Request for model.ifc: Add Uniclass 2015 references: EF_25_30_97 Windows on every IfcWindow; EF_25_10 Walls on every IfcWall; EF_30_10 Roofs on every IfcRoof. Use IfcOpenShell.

First a look at what the model holds.

```python
import ifcopenshell

model = ifcopenshell.open("model.ifc")
print(model.schema)
print("classifications:", [c.Name for c in model.by_type("IfcClassification")])
for ifc_class in ("IfcDoor", "IfcRoof", "IfcStair", "IfcWall", "IfcWindow"):
    print(ifc_class, len(model.by_type(ifc_class)))
```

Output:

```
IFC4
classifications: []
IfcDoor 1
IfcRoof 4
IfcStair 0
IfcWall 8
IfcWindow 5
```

```python
import ifcopenshell
import ifcopenshell.api.classification

model = ifcopenshell.open("model.ifc")

system = ifcopenshell.api.classification.add_classification(model, classification="Uniclass 2015")

codes = {
    "IfcWindow": ("EF_25_30_97", "Windows"),
    "IfcWall": ("EF_25_10", "Walls"),
    "IfcRoof": ("EF_30_10", "Roofs"),
}
for ifc_class, (code, name) in codes.items():
    products = model.by_type(ifc_class)
    ifcopenshell.api.classification.add_reference(
        model, products=products, classification=system, identification=code, name=name
    )
    print(code, len(products))

model.write("model_rev.ifc")
```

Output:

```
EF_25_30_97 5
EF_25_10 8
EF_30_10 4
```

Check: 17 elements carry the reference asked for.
